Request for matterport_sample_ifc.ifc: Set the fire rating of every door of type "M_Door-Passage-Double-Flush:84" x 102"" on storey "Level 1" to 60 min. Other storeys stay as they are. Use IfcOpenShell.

First a look at what the model holds.

```python
import ifcopenshell
import ifcopenshell.util.element

model = ifcopenshell.open("matterport_sample_ifc.ifc")
print(model.schema)
storey = next(s for s in model.by_type("IfcBuildingStorey") if s.Name == "Level 1")
doors = [e for e in ifcopenshell.util.element.get_decomposition(storey) if e.is_a("IfcDoor")]
seen = {}
for e in doors:
    element_type = ifcopenshell.util.element.get_type(e)
    key = (element_type.Name if element_type != e and element_type else None, ifcopenshell.util.element.get_pset(e, "Pset_DoorCommon", "FireRating"))
    seen[key] = seen.get(key, 0) + 1
for (name, value), count in sorted(seen.items(), key=str):
    print(count, "x", name, "|", value)
```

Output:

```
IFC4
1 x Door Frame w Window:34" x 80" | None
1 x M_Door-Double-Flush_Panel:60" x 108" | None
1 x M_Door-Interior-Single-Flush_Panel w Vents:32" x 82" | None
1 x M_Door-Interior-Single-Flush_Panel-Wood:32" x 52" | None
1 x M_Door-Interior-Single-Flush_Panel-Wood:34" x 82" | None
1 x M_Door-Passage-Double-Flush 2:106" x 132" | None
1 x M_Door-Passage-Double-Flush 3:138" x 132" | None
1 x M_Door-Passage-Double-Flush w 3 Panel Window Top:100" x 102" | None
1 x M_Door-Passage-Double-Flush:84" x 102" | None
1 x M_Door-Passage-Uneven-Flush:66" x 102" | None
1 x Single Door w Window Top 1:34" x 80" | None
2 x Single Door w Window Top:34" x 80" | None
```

```python
import ifcopenshell
import ifcopenshell.api.pset
import ifcopenshell.util.element

model = ifcopenshell.open("matterport_sample_ifc.ifc")

storey = next(s for s in model.by_type("IfcBuildingStorey") if s.Name == "Level 1")
doors = [e for e in ifcopenshell.util.element.get_decomposition(storey) if e.is_a("IfcDoor")]

count = 0
for e in doors:
    element_type = ifcopenshell.util.element.get_type(e)
    if element_type in (None, e) or element_type.Name != 'M_Door-Passage-Double-Flush:84" x 102"':
        continue
    # add_pset returns the element's existing set when there is one.
    pset = ifcopenshell.api.pset.add_pset(model, product=e, name="Pset_DoorCommon")
    ifcopenshell.api.pset.edit_pset(model, pset=pset, properties={"FireRating": "60 min"})
    count += 1

print(count, "doors updated")

model.write("matterport_sample_ifc_edited.ifc")
```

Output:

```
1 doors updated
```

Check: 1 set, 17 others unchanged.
